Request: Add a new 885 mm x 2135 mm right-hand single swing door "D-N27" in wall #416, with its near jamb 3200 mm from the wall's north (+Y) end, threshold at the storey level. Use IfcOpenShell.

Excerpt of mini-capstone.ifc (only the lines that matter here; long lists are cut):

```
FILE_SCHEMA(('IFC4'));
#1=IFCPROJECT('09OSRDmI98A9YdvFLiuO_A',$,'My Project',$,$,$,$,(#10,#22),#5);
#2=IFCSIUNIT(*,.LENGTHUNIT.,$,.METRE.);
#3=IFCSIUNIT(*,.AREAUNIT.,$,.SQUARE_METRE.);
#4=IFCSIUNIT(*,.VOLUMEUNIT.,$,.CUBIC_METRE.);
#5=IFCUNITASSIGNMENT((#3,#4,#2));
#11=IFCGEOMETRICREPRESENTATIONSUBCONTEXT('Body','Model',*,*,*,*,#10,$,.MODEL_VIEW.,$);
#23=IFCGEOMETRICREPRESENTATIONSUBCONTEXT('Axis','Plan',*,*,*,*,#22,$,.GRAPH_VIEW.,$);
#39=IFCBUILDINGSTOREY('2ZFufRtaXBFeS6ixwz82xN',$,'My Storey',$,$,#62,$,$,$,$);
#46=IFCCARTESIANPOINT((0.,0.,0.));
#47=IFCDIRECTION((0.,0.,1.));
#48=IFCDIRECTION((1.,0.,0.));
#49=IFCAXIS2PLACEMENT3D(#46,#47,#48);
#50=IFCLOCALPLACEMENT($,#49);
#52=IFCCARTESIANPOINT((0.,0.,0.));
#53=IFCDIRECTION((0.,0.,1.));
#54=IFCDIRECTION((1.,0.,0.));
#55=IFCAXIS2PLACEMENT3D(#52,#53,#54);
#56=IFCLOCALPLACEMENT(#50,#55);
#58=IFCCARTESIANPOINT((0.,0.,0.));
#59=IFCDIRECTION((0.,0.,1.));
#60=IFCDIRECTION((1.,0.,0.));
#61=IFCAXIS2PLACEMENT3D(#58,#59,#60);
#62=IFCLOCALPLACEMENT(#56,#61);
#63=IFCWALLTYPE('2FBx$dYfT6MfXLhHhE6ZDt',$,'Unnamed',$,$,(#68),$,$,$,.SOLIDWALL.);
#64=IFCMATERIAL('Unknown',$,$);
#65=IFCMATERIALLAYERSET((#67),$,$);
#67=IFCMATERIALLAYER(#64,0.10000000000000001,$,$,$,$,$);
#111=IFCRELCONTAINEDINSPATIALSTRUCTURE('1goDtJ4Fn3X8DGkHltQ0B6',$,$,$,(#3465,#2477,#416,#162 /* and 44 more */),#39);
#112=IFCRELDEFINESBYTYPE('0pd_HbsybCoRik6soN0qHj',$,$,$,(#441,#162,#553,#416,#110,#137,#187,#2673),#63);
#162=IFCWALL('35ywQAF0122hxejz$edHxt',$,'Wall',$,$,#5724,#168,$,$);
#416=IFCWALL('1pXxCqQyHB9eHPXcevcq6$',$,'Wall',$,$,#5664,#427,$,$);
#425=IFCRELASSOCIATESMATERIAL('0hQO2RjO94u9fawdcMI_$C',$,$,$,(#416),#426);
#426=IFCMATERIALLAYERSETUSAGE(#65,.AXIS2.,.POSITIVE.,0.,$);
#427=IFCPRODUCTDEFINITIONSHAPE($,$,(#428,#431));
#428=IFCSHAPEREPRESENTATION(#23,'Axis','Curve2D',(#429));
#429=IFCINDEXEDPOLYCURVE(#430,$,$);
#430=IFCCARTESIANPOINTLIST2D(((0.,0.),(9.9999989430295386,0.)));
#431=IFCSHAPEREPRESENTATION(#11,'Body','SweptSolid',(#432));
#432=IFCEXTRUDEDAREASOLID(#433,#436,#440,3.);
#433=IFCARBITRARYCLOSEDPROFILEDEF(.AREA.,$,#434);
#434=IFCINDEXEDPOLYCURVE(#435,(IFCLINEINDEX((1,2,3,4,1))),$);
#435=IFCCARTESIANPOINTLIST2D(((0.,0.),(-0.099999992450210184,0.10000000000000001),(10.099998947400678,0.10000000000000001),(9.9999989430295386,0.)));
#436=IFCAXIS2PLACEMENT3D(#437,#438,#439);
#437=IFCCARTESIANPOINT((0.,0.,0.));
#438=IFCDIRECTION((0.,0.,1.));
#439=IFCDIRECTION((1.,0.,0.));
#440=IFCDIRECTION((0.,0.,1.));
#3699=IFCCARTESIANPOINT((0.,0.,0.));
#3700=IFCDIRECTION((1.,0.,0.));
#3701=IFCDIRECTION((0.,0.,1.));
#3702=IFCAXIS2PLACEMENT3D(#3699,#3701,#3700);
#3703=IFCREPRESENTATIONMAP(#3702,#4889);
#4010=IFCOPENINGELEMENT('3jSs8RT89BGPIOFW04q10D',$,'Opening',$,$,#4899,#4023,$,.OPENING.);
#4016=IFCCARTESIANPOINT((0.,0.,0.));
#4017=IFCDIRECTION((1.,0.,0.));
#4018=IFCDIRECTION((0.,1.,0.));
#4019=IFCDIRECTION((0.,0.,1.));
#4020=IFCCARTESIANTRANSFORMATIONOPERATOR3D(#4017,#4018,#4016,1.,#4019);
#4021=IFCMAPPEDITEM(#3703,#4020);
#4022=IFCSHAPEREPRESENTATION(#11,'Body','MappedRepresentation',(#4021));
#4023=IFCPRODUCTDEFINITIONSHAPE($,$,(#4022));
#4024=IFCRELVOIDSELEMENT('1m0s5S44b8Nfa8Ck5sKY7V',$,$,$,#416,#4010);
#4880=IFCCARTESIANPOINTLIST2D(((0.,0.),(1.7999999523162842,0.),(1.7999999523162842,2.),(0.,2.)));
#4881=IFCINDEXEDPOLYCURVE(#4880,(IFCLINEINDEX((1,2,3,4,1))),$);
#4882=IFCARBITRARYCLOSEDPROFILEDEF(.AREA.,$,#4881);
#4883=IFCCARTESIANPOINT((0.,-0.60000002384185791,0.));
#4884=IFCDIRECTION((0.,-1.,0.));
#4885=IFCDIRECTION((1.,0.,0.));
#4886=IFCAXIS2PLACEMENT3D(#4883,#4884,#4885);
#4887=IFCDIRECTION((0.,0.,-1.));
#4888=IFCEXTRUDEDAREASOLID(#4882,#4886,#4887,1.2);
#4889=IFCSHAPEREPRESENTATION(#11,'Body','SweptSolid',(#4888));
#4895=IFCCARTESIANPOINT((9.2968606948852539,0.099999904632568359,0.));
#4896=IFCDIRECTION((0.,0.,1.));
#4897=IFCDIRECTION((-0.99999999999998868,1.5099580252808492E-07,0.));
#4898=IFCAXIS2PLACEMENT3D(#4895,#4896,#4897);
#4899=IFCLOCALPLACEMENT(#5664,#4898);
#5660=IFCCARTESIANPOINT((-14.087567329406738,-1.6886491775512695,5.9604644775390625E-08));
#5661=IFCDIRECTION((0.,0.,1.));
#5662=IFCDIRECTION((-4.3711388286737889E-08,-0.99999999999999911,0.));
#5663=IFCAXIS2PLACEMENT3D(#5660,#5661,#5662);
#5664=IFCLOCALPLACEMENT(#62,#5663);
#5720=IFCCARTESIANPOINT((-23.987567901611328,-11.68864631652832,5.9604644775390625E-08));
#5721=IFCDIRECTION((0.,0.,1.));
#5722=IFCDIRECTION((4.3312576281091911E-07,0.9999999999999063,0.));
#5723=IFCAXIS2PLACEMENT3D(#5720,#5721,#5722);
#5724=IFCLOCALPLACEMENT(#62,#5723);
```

```python
import numpy as np
import ifcopenshell
import ifcopenshell.api.feature
import ifcopenshell.api.geometry
import ifcopenshell.api.root
import ifcopenshell.api.spatial
import ifcopenshell.geom
import ifcopenshell.util.element
import ifcopenshell.util.placement
import ifcopenshell.util.representation
import ifcopenshell.util.shape
import ifcopenshell.util.unit

model = ifcopenshell.open("mini-capstone.ifc")
unit_scale = ifcopenshell.util.unit.calculate_unit_scale(model)
settings = ifcopenshell.geom.settings()


def volume(element):
    """Net volume in cubic metres, openings subtracted."""
    shape = ifcopenshell.geom.create_shape(settings, element)
    return ifcopenshell.util.shape.get_volume(shape.geometry)


wall = model.by_guid("1pXxCqQyHB9eHPXcevcq6$")
storey = ifcopenshell.util.element.get_container(wall, ifc_class="IfcBuildingStorey")
context = ifcopenshell.util.representation.get_context(model, "Model", "Body", "MODEL_VIEW")
before = volume(wall)

width, height, from_end, sill = 0.885, 2.135, 3.2, 0.0  # metres

# The wall runs along its own X axis, and the end named is its -X end.
wall_shape = ifcopenshell.geom.create_shape(settings, wall)
x, y, z = ifcopenshell.util.shape.get_vertices(wall_shape.geometry).T
start = x.min() + from_end
face, thickness = float(y.min()), float(y.max() - y.min())
wall_matrix = ifcopenshell.util.placement.get_local_placement(wall.ObjectPlacement)
level = ifcopenshell.util.placement.get_local_placement(storey.ObjectPlacement)[2, 3]


def in_wall(x, y):
    """Placement at x, y metres in the wall's axes, at sill height."""
    matrix = wall_matrix.copy()
    matrix[:, 3] = wall_matrix @ np.array([x / unit_scale, y / unit_scale, 0.0, 1.0])
    matrix[2, 3] = level + sill / unit_scale
    return matrix


# Opening: a box that overshoots both wall faces by 50 mm.
opening = ifcopenshell.api.root.create_entity(model, ifc_class="IfcOpeningElement", predefined_type="OPENING")
box = ifcopenshell.api.geometry.add_wall_representation(
    model, context=context, length=width, height=height, thickness=thickness + 0.1
)
ifcopenshell.api.geometry.assign_representation(model, product=opening, representation=box)
ifcopenshell.api.geometry.edit_object_placement(model, product=opening, matrix=in_wall(start, face - 0.05), is_si=False)
ifcopenshell.api.feature.add_feature(model, feature=opening, element=wall)

door = ifcopenshell.api.root.create_entity(model, ifc_class="IfcDoor", name="D-N27", predefined_type="DOOR")
door.OverallWidth, door.OverallHeight = width / unit_scale, height / unit_scale
door.OperationType = "SINGLE_SWING_RIGHT"
body = ifcopenshell.api.geometry.add_door_representation(
    model,
    context=context,
    overall_width=door.OverallWidth,
    overall_height=door.OverallHeight,
    operation_type="SINGLE_SWING_RIGHT",
    lining_properties={"LiningDepth": thickness / unit_scale, "ThresholdDepth": thickness / unit_scale},
)
ifcopenshell.api.geometry.assign_representation(model, product=door, representation=body)
ifcopenshell.api.spatial.assign_container(model, products=[door], relating_structure=storey)
ifcopenshell.api.feature.add_filling(model, opening=opening, element=door)

# The lining spans the wall, so the door starts at the wall face.
ifcopenshell.api.geometry.edit_object_placement(model, product=door, matrix=in_wall(start, face), is_si=False)

after = volume(wall)

print(f"wall volume {before:.3f} -> {after:.3f} m3")

model.write("mini-capstone_v2.ifc")
```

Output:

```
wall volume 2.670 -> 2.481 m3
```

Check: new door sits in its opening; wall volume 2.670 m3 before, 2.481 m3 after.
